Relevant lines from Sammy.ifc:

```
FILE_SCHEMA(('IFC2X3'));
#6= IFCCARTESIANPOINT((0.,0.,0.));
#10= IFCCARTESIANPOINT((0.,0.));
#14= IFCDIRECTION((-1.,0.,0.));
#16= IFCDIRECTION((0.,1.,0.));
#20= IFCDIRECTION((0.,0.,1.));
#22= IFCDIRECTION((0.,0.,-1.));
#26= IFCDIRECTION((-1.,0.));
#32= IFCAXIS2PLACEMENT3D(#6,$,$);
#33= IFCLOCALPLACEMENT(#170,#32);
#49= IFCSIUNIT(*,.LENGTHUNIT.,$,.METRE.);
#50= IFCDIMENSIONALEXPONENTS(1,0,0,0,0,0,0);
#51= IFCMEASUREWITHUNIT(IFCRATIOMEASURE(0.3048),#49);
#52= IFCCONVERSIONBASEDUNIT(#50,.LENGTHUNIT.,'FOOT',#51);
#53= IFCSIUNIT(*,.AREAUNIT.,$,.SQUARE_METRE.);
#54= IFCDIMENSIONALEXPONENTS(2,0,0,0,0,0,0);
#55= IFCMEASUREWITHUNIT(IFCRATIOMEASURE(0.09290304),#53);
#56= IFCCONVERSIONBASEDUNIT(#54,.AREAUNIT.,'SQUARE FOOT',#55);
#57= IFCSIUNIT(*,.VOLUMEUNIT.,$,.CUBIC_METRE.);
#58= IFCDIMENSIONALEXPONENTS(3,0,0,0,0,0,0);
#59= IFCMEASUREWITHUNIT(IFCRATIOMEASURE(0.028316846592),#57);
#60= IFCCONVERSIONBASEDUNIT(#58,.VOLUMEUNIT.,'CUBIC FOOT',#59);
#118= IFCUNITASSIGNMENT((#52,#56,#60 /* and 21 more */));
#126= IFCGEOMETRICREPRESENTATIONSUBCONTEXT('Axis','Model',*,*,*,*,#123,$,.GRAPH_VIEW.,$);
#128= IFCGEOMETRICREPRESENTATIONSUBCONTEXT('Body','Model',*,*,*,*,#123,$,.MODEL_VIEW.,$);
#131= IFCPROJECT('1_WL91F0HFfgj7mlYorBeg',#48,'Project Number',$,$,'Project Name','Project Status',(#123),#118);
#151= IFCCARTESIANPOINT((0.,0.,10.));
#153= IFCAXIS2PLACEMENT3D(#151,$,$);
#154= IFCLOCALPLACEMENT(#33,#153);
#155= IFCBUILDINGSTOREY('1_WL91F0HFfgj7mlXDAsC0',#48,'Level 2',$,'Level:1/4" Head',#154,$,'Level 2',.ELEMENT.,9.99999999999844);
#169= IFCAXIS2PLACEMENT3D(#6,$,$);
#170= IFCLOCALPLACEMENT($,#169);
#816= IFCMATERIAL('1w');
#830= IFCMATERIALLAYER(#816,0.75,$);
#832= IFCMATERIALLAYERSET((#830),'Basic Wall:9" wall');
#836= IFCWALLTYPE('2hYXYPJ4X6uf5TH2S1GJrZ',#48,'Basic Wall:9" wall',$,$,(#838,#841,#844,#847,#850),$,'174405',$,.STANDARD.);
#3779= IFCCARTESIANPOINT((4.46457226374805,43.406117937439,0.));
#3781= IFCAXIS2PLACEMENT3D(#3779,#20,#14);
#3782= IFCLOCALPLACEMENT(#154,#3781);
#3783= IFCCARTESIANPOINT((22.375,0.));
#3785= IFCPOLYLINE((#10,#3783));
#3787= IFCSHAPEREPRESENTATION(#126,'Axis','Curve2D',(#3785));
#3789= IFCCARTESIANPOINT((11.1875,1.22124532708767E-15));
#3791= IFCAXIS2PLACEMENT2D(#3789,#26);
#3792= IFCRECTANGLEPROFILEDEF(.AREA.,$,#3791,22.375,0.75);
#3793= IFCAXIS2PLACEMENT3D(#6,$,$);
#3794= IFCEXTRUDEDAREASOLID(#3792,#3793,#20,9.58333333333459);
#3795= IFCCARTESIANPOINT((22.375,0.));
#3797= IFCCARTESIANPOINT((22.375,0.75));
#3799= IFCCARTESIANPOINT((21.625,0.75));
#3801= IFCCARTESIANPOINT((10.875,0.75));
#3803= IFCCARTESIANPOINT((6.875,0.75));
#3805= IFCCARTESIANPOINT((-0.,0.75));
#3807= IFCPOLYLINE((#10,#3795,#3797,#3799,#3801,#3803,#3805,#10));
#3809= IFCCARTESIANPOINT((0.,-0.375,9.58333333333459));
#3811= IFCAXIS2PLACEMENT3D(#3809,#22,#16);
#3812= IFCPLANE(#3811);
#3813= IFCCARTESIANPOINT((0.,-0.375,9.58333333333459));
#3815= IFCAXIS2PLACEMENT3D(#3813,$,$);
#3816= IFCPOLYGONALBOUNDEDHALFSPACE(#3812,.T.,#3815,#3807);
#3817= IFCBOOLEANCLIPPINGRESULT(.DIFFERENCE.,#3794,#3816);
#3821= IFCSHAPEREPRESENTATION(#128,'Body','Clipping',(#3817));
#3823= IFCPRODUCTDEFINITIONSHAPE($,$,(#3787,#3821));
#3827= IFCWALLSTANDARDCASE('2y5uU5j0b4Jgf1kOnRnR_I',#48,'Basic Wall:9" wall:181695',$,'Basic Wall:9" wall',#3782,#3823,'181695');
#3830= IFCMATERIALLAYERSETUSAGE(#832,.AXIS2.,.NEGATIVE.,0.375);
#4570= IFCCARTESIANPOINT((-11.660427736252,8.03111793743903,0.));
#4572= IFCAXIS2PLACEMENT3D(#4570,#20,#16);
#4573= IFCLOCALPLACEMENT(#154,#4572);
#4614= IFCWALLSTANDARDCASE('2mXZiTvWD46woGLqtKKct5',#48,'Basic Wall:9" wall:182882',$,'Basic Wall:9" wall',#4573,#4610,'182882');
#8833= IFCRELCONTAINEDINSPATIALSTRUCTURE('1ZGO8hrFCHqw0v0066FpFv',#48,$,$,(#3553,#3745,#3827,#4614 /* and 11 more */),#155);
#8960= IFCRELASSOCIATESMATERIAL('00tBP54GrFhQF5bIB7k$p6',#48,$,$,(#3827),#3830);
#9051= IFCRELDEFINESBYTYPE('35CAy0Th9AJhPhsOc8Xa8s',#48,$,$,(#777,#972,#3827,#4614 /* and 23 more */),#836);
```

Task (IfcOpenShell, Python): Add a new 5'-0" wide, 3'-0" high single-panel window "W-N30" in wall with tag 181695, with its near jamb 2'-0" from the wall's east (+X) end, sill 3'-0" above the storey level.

```python
import numpy as np
import ifcopenshell
import ifcopenshell.api.feature
import ifcopenshell.api.geometry
import ifcopenshell.api.root
import ifcopenshell.api.spatial
import ifcopenshell.api.type
import ifcopenshell.geom
import ifcopenshell.util.element
import ifcopenshell.util.placement
import ifcopenshell.util.representation
import ifcopenshell.util.shape
import ifcopenshell.util.unit

model = ifcopenshell.open("Sammy.ifc")
unit_scale = ifcopenshell.util.unit.calculate_unit_scale(model)
settings = ifcopenshell.geom.settings()


def volume(element):
    """Net volume in cubic metres, openings subtracted."""
    shape = ifcopenshell.geom.create_shape(settings, element)
    return ifcopenshell.util.shape.get_volume(shape.geometry)


wall = model.by_guid("2y5uU5j0b4Jgf1kOnRnR_I")
storey = ifcopenshell.util.element.get_container(wall, ifc_class="IfcBuildingStorey")
context = ifcopenshell.util.representation.get_context(model, "Model", "Body", "MODEL_VIEW")
before = volume(wall)

width, height, from_end, sill = 1.524, 0.9144, 0.6096, 0.9144  # metres

# The wall runs along its own X axis, and the end named is its -X end.
wall_shape = ifcopenshell.geom.create_shape(settings, wall)
x, y, z = ifcopenshell.util.shape.get_vertices(wall_shape.geometry).T
start = x.min() + from_end
face, thickness = float(y.min()), float(y.max() - y.min())
wall_matrix = ifcopenshell.util.placement.get_local_placement(wall.ObjectPlacement)
level = ifcopenshell.util.placement.get_local_placement(storey.ObjectPlacement)[2, 3]


def in_wall(x, y):
    """Placement at x, y metres in the wall's axes, at sill height."""
    matrix = wall_matrix.copy()
    matrix[:, 3] = wall_matrix @ np.array([x / unit_scale, y / unit_scale, 0.0, 1.0])
    matrix[2, 3] = level + sill / unit_scale
    return matrix


# Opening: a box that overshoots both wall faces by 50 mm.
opening = ifcopenshell.api.root.create_entity(model, ifc_class="IfcOpeningElement")
box = ifcopenshell.api.geometry.add_wall_representation(
    model, context=context, length=width, height=height, thickness=thickness + 0.1
)
ifcopenshell.api.geometry.assign_representation(model, product=opening, representation=box)
ifcopenshell.api.geometry.edit_object_placement(model, product=opening, matrix=in_wall(start, face - 0.05), is_si=False)
ifcopenshell.api.feature.add_feature(model, feature=opening, element=wall)

window = ifcopenshell.api.root.create_entity(model, ifc_class="IfcWindow", name="W-N30")
window.OverallWidth, window.OverallHeight = width / unit_scale, height / unit_scale
body = ifcopenshell.api.geometry.add_window_representation(
    model,
    context=context,
    overall_width=window.OverallWidth,
    overall_height=window.OverallHeight,
    partition_type="SINGLE_PANEL",
)
ifcopenshell.api.geometry.assign_representation(model, product=window, representation=body)
ifcopenshell.api.spatial.assign_container(model, products=[window], relating_structure=storey)
fills = ifcopenshell.api.feature.add_filling(model, opening=opening, element=window)
fills.OwnerHistory = window.OwnerHistory  # required in IFC2X3

# IFC2X3 keeps the operation on the window style.
style = ifcopenshell.api.root.create_entity(model, ifc_class="IfcWindowStyle", name="W-N30")
style.OperationType, style.ConstructionType = "SINGLE_PANEL", "NOTDEFINED"
style.ParameterTakesPrecedence = style.Sizeable = False
ifcopenshell.api.type.assign_type(model, related_objects=[window], relating_type=style)

# Centre the window in the wall's thickness.
ifcopenshell.api.geometry.edit_object_placement(model, product=window, matrix=in_wall(start, face), is_si=False)
window_shape = ifcopenshell.geom.create_shape(settings, window)
depth = ifcopenshell.util.shape.get_vertices(window_shape.geometry)[:, 1]
offset = face + thickness / 2 - (depth.min() + depth.max()) / 2
ifcopenshell.api.geometry.edit_object_placement(model, product=window, matrix=in_wall(start, offset), is_si=False)

after = volume(wall)

print(f"wall volume {before:.3f} -> {after:.3f} m3")

model.write("Sammy_rev.ifc")
```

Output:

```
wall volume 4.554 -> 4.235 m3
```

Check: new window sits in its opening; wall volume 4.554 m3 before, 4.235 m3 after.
